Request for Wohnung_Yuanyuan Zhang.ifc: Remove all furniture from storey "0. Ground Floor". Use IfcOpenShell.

First a look at what the model holds.

```python
import ifcopenshell
import ifcopenshell.util.element

model = ifcopenshell.open("Wohnung_Yuanyuan Zhang.ifc")
print(model.schema)
storey = next(s for s in model.by_type("IfcBuildingStorey") if s.Name == "0. Ground Floor")
furniture = [e for e in ifcopenshell.util.element.get_decomposition(storey) if e.is_a("IfcFurnishingElement")]
seen = {}
for e in furniture:
    element_type = ifcopenshell.util.element.get_type(e)
    name = element_type.Name if element_type not in (None, e) else None
    seen[name] = seen.get(name, 0) + 1
for name, count in sorted(seen.items(), key=str):
    print(count, "x", name)
```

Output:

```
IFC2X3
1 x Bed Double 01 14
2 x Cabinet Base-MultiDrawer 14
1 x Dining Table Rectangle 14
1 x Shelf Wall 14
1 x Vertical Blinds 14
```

```python
import ifcopenshell
import ifcopenshell.api.root
import ifcopenshell.util.element

model = ifcopenshell.open("Wohnung_Yuanyuan Zhang.ifc")

storey = next(s for s in model.by_type("IfcBuildingStorey") if s.Name == "0. Ground Floor")
furniture = [e for e in ifcopenshell.util.element.get_decomposition(storey) if e.is_a("IfcFurnishingElement")]

for e in furniture:
    ifcopenshell.api.root.remove_product(model, product=e)
print(len(furniture), "removed")

model.write("Wohnung_Yuanyuan Zhang_v2.ifc")
```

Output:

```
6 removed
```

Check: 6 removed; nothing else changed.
